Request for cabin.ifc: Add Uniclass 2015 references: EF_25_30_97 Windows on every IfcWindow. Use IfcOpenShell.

First a look at what the model holds.

```python
import ifcopenshell

model = ifcopenshell.open("cabin.ifc")
print(model.schema)
print("classifications:", [c.Name for c in model.by_type("IfcClassification")])
for ifc_class in ("IfcDoor", "IfcRoof", "IfcStair", "IfcWall", "IfcWindow"):
    print(ifc_class, len(model.by_type(ifc_class)))
```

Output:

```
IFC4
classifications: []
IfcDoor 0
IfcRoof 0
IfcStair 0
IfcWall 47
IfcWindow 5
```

```python
import ifcopenshell
import ifcopenshell.api.classification

model = ifcopenshell.open("cabin.ifc")

system = ifcopenshell.api.classification.add_classification(model, classification="Uniclass 2015")

codes = {
    "IfcWindow": ("EF_25_30_97", "Windows"),
}
for ifc_class, (code, name) in codes.items():
    products = model.by_type(ifc_class)
    ifcopenshell.api.classification.add_reference(
        model, products=products, classification=system, identification=code, name=name
    )
    print(code, len(products))

model.write("cabin_rev.ifc")
```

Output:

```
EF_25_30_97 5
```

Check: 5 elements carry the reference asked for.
